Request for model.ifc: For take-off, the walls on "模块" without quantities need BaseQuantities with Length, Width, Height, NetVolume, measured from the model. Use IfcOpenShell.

First a look at what the model holds.

```python
import ifcopenshell
import ifcopenshell.util.element
import ifcopenshell.util.unit

model = ifcopenshell.open("model.ifc")
print(model.schema)
for unit_type in ("LENGTHUNIT", "AREAUNIT", "VOLUMEUNIT"):
    print(unit_type, ifcopenshell.util.unit.calculate_unit_scale(model, unit_type))
storey = next(s for s in model.by_type("IfcBuildingStorey") if s.Name == "模块")
walls = [e for e in ifcopenshell.util.element.get_decomposition(storey) if e.is_a("IfcWall")]
for e in sorted(walls, key=lambda e: e.id()):
    print(e.id(), e.is_a(), e.Name, list(ifcopenshell.util.element.get_psets(e, qtos_only=True)), sep=" | ")
```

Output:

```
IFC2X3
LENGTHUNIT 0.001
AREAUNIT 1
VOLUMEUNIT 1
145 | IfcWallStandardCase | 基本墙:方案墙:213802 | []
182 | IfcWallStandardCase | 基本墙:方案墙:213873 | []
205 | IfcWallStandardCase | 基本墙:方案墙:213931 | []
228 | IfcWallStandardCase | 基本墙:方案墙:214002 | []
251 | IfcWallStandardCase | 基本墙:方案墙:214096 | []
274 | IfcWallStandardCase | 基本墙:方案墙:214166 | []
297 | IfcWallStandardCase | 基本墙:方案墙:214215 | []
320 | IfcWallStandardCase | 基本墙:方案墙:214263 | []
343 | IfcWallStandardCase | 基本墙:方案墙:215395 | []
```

```python
import ifcopenshell
import ifcopenshell.api.pset
import ifcopenshell.geom
import ifcopenshell.util.element
import ifcopenshell.util.shape
import ifcopenshell.util.unit

model = ifcopenshell.open("model.ifc")
unit_scale = ifcopenshell.util.unit.calculate_unit_scale(model)
volume_scale = ifcopenshell.util.unit.calculate_unit_scale(model, "VOLUMEUNIT")
settings = ifcopenshell.geom.settings()

storey = next(s for s in model.by_type("IfcBuildingStorey") if s.Name == "模块")
walls = [e for e in ifcopenshell.util.element.get_decomposition(storey) if e.is_a("IfcWall")]

for e in sorted(walls, key=lambda e: e.id()):
    if ifcopenshell.util.element.get_psets(e, qtos_only=True, should_inherit=False):
        continue
    # Geometry comes back in metres, in the element's own axes.
    shape = ifcopenshell.geom.create_shape(settings, e)
    values = {
        "Length": ifcopenshell.util.shape.get_x(shape.geometry) / unit_scale,
        "Width": ifcopenshell.util.shape.get_y(shape.geometry) / unit_scale,
        "Height": ifcopenshell.util.shape.get_z(shape.geometry) / unit_scale,
        "NetVolume": ifcopenshell.util.shape.get_volume(shape.geometry) / volume_scale,
    }
    qto = ifcopenshell.api.pset.add_qto(model, product=e, name="BaseQuantities")
    ifcopenshell.api.pset.edit_qto(model, qto=qto, properties=values)
    print(e.id(), {k: round(v, 3) for k, v in values.items()})

model.write("model_v2.ifc")
```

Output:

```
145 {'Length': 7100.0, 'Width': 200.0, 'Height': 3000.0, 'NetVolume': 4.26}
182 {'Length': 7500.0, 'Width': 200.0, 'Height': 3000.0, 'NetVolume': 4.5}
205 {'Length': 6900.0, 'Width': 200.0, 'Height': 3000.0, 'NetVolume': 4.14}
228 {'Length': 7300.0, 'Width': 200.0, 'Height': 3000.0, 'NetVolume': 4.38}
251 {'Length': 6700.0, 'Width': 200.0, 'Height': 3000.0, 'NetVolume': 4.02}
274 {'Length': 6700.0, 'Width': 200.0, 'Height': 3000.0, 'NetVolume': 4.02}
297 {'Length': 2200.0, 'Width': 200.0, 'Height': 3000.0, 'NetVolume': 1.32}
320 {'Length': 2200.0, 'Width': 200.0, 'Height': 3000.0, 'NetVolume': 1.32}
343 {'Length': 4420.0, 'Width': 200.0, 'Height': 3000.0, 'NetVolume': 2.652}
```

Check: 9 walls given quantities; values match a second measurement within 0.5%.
